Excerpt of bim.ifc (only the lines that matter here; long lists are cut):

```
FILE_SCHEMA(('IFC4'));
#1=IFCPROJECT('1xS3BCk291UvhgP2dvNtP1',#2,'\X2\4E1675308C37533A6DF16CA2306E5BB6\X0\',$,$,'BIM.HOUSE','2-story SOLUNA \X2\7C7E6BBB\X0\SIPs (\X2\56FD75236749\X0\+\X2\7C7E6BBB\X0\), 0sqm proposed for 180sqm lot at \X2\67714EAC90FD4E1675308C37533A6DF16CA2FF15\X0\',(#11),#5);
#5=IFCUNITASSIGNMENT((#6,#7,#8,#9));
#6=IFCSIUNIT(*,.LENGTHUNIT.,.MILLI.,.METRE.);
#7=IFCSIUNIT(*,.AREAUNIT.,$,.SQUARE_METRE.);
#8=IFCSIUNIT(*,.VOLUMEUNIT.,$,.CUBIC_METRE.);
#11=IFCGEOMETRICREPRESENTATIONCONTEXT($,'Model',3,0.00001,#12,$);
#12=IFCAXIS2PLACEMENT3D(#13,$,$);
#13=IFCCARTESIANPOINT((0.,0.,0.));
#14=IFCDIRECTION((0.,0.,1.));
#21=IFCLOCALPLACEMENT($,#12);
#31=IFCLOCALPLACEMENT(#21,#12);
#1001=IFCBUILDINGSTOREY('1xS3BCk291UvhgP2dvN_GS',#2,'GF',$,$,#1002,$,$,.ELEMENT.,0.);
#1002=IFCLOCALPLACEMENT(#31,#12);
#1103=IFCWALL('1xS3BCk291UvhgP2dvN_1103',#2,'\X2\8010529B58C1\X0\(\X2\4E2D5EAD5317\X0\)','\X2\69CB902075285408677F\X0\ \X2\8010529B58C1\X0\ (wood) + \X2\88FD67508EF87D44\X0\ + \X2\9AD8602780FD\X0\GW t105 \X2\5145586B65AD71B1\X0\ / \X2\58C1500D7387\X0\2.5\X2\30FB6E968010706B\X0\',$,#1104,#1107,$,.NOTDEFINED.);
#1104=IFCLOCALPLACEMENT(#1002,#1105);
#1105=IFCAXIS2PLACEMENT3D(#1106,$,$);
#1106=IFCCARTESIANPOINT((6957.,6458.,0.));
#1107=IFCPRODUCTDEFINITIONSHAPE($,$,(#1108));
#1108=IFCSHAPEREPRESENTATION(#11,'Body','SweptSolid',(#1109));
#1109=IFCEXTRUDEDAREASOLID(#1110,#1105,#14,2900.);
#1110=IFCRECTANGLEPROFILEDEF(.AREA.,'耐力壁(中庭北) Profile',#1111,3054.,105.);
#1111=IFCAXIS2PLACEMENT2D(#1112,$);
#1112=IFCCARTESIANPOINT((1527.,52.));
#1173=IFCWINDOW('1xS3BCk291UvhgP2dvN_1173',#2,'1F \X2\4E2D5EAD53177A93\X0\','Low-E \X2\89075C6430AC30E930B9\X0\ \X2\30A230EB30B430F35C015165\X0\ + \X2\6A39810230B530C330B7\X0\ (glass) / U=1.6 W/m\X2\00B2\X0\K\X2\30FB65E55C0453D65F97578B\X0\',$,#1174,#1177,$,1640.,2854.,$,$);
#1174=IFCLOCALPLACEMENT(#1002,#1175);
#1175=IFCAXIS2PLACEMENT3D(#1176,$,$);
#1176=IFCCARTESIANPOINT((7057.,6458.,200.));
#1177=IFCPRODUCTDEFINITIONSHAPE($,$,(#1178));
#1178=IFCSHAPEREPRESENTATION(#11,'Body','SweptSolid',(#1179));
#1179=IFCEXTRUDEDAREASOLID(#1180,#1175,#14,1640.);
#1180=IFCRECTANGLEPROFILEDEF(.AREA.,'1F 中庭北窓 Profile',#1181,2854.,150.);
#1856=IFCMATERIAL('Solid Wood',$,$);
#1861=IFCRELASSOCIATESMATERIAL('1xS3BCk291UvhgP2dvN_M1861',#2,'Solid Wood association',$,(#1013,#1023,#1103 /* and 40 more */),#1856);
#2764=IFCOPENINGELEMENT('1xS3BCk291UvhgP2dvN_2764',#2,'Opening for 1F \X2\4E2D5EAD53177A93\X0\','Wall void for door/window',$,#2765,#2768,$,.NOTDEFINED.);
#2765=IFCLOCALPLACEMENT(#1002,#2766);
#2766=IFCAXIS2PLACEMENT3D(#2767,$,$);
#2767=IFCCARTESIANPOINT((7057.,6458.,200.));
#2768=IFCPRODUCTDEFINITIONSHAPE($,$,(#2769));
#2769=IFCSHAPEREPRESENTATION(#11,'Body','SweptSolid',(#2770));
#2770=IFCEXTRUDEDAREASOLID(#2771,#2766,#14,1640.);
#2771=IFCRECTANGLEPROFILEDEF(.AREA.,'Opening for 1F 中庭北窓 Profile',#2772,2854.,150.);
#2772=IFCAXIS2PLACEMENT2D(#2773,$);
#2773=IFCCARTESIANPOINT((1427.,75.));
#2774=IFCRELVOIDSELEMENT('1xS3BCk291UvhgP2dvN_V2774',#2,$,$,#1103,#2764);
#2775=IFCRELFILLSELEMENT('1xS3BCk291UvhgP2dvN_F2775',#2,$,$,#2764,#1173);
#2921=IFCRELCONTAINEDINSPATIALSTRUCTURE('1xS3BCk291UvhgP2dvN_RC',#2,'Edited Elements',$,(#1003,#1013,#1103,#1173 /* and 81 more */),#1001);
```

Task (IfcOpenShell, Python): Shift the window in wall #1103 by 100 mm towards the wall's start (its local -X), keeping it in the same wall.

```python
import ifcopenshell
import ifcopenshell.api.geometry
import ifcopenshell.util.placement

model = ifcopenshell.open("bim.ifc")

window = model.by_guid("1xS3BCk291UvhgP2dvN_1173")
opening = window.FillsVoids[0].RelatingOpeningElement
wall = opening.VoidsElements[0].RelatingBuildingElement

wall_matrix = ifcopenshell.util.placement.get_local_placement(wall.ObjectPlacement)
shift = wall_matrix[:3, 0] * -100.0
before = ifcopenshell.util.placement.get_local_placement(window.ObjectPlacement)[:3, 3].copy()

# The window is not placed relative to its opening, so move both.
for product in (opening, window):
    matrix = ifcopenshell.util.placement.get_local_placement(product.ObjectPlacement)
    matrix[:3, 3] += shift
    ifcopenshell.api.geometry.edit_object_placement(model, product=product, matrix=matrix, is_si=False)

after = ifcopenshell.util.placement.get_local_placement(window.ObjectPlacement)[:3, 3]
print("window moved by", (after - before).round(3) + 0.0)

model.write("bim_updated.ifc")
```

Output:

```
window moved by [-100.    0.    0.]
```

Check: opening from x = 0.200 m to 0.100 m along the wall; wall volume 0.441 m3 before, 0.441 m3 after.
